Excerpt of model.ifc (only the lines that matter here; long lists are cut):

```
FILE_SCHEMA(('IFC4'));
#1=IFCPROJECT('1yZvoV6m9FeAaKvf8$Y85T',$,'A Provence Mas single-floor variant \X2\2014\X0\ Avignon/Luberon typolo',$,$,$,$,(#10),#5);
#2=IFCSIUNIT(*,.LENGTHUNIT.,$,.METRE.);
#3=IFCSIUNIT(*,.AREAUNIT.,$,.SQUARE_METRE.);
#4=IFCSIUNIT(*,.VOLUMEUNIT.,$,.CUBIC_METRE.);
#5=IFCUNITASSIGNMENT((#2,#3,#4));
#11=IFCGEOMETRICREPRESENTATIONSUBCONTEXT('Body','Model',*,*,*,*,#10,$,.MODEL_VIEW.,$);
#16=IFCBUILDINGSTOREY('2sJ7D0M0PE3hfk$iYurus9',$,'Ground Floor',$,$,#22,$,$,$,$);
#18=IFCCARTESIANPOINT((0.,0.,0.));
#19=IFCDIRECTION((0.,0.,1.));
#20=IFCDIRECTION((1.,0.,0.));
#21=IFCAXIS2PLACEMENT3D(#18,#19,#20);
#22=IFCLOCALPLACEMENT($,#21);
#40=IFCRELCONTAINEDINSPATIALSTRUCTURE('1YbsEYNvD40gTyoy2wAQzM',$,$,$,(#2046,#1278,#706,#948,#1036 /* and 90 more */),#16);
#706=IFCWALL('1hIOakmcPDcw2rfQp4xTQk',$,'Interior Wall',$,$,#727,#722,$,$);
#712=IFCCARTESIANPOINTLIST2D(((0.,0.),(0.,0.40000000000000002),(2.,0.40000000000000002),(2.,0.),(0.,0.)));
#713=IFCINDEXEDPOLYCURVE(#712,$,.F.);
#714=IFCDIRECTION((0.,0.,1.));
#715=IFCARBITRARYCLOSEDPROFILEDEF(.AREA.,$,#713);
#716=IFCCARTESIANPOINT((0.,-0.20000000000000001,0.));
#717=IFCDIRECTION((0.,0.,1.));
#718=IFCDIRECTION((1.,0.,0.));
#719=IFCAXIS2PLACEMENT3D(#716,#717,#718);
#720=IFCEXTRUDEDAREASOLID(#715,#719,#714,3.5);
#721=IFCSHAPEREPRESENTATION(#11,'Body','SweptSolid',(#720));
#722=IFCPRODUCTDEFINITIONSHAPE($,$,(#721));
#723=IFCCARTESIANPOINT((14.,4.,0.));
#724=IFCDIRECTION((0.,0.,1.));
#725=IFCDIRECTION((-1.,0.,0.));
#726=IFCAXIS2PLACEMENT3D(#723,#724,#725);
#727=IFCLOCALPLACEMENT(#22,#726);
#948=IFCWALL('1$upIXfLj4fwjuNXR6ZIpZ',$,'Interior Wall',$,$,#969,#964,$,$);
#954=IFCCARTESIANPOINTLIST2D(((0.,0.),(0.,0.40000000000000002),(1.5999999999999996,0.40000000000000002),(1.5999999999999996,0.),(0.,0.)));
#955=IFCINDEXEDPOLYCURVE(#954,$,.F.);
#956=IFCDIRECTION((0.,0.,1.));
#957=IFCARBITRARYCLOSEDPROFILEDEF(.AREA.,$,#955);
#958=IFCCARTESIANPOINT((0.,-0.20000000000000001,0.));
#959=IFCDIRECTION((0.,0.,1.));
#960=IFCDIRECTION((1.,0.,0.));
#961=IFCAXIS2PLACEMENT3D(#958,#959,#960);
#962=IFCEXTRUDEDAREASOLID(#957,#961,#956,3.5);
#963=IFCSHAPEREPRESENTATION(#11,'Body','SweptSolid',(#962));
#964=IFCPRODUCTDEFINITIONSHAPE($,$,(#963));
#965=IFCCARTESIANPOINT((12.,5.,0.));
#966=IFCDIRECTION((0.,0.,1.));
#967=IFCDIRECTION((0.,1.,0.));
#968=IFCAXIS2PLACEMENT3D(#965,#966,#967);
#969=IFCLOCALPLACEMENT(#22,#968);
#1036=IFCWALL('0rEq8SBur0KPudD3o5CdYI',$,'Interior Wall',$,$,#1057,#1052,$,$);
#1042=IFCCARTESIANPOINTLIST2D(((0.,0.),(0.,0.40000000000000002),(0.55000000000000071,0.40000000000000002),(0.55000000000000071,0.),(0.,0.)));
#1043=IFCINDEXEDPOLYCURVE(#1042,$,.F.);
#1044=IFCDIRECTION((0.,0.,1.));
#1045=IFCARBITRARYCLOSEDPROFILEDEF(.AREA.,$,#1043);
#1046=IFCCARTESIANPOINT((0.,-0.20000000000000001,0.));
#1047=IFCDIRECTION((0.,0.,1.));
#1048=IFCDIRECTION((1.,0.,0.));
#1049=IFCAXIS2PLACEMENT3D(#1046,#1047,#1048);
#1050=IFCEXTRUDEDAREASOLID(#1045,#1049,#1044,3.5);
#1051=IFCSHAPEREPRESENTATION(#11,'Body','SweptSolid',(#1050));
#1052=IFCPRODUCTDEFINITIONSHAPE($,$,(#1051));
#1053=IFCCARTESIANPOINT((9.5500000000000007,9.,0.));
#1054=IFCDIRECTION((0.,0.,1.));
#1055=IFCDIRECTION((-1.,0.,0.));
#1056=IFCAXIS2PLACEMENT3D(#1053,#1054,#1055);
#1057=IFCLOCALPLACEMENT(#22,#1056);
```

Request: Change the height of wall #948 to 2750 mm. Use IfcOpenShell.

```python
import ifcopenshell
import ifcopenshell.geom
import ifcopenshell.util.representation
import ifcopenshell.util.shape

model = ifcopenshell.open("model.ifc")
settings = ifcopenshell.geom.settings()


def volume(element):
    """Net volume in cubic metres, openings subtracted."""
    shape = ifcopenshell.geom.create_shape(settings, element)
    return ifcopenshell.util.shape.get_volume(shape.geometry)


wall = model.by_id(948)
before = volume(wall)

body = ifcopenshell.util.representation.get_representation(wall, "Model", "Body")
solid = body.Items[0]
old_height = solid.Depth
solid.Depth = 2.75
after = volume(wall)

print(f"height {old_height:g} -> {solid.Depth:g}, volume {before:.3f} -> {after:.3f} m3")

model.write("model_updated.ifc")
```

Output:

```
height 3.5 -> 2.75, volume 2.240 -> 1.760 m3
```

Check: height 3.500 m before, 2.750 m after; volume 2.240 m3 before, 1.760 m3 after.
